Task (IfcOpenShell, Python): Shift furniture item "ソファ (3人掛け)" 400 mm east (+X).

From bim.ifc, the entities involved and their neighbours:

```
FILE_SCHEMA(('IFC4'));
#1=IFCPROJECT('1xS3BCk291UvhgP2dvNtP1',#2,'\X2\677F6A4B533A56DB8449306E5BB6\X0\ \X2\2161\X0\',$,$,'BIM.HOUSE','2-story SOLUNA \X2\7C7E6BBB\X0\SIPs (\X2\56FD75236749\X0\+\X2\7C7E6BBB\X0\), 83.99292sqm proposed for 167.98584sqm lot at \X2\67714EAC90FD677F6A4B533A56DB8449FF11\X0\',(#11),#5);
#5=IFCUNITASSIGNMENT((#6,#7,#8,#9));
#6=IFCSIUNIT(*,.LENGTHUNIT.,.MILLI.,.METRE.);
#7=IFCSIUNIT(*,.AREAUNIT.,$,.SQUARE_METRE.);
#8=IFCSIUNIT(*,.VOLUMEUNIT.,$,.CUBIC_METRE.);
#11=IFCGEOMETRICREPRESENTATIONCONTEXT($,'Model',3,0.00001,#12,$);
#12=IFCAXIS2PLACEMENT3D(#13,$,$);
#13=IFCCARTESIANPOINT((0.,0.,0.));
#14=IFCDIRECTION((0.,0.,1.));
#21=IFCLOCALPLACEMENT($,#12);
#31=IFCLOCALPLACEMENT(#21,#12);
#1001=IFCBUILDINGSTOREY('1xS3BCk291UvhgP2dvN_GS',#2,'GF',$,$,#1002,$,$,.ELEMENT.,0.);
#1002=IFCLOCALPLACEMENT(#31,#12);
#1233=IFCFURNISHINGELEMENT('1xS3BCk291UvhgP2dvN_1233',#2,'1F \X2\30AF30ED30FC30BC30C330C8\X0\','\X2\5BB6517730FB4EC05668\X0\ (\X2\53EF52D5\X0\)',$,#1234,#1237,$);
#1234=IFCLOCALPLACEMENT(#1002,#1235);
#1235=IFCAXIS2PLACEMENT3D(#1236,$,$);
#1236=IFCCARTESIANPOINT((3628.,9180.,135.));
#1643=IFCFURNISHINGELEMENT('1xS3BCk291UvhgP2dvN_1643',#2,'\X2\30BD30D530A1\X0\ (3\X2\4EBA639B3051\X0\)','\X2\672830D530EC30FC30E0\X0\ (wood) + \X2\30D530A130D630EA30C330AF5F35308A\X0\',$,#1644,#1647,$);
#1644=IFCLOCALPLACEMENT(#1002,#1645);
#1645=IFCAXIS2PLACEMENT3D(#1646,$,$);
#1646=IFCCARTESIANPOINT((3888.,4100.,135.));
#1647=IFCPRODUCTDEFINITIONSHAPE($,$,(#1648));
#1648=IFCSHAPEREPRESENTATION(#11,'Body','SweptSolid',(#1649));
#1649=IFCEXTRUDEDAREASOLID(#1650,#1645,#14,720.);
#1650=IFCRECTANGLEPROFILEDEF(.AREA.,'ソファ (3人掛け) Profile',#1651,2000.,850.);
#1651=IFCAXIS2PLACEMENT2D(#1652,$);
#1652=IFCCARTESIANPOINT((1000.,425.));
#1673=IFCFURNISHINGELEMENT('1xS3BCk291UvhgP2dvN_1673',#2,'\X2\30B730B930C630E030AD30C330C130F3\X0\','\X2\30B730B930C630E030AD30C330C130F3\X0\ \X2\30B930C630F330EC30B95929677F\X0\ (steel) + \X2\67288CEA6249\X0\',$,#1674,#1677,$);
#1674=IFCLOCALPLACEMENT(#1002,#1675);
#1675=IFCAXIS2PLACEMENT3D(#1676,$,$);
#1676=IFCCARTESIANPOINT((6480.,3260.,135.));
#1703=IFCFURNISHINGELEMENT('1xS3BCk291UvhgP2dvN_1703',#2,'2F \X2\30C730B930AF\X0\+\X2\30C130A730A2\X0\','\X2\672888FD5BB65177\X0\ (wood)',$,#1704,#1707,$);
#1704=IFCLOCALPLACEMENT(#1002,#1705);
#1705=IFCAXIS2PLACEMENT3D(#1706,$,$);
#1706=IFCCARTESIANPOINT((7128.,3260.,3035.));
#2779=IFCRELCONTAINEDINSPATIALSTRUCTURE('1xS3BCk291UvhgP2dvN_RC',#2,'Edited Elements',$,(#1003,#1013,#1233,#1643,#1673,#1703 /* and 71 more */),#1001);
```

```python
import ifcopenshell
import ifcopenshell.api.geometry
import ifcopenshell.util.placement

model = ifcopenshell.open("bim.ifc")

item = model.by_guid("1xS3BCk291UvhgP2dvN_1643")
matrix = ifcopenshell.util.placement.get_local_placement(item.ObjectPlacement)
matrix[0, 3] += 400.0
ifcopenshell.api.geometry.edit_object_placement(model, product=item, matrix=matrix, is_si=False)

print(ifcopenshell.util.placement.get_local_placement(item.ObjectPlacement).round(3) + 0.0)

model.write("bim_v2.ifc")
```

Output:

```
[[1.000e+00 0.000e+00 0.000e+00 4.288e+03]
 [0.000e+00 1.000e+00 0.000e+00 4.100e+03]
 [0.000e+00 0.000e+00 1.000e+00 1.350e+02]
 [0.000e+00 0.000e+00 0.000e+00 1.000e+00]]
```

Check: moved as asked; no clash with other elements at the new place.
